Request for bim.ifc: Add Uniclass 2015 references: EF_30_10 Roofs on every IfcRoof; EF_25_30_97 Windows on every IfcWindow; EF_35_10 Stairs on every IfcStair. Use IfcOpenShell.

First a look at what the model holds.

```python
import ifcopenshell

model = ifcopenshell.open("bim.ifc")
print(model.schema)
print("classifications:", [c.Name for c in model.by_type("IfcClassification")])
for ifc_class in ("IfcDoor", "IfcRoof", "IfcStair", "IfcWall", "IfcWindow"):
    print(ifc_class, len(model.by_type(ifc_class)))
```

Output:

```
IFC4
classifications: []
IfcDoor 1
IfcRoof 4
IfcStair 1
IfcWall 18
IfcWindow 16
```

```python
import ifcopenshell
import ifcopenshell.api.classification

model = ifcopenshell.open("bim.ifc")

system = ifcopenshell.api.classification.add_classification(model, classification="Uniclass 2015")

codes = {
    "IfcRoof": ("EF_30_10", "Roofs"),
    "IfcWindow": ("EF_25_30_97", "Windows"),
    "IfcStair": ("EF_35_10", "Stairs"),
}
for ifc_class, (code, name) in codes.items():
    products = model.by_type(ifc_class)
    ifcopenshell.api.classification.add_reference(
        model, products=products, classification=system, identification=code, name=name
    )
    print(code, len(products))

model.write("bim_updated.ifc")
```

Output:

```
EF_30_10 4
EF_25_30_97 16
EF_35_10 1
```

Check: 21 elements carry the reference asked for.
